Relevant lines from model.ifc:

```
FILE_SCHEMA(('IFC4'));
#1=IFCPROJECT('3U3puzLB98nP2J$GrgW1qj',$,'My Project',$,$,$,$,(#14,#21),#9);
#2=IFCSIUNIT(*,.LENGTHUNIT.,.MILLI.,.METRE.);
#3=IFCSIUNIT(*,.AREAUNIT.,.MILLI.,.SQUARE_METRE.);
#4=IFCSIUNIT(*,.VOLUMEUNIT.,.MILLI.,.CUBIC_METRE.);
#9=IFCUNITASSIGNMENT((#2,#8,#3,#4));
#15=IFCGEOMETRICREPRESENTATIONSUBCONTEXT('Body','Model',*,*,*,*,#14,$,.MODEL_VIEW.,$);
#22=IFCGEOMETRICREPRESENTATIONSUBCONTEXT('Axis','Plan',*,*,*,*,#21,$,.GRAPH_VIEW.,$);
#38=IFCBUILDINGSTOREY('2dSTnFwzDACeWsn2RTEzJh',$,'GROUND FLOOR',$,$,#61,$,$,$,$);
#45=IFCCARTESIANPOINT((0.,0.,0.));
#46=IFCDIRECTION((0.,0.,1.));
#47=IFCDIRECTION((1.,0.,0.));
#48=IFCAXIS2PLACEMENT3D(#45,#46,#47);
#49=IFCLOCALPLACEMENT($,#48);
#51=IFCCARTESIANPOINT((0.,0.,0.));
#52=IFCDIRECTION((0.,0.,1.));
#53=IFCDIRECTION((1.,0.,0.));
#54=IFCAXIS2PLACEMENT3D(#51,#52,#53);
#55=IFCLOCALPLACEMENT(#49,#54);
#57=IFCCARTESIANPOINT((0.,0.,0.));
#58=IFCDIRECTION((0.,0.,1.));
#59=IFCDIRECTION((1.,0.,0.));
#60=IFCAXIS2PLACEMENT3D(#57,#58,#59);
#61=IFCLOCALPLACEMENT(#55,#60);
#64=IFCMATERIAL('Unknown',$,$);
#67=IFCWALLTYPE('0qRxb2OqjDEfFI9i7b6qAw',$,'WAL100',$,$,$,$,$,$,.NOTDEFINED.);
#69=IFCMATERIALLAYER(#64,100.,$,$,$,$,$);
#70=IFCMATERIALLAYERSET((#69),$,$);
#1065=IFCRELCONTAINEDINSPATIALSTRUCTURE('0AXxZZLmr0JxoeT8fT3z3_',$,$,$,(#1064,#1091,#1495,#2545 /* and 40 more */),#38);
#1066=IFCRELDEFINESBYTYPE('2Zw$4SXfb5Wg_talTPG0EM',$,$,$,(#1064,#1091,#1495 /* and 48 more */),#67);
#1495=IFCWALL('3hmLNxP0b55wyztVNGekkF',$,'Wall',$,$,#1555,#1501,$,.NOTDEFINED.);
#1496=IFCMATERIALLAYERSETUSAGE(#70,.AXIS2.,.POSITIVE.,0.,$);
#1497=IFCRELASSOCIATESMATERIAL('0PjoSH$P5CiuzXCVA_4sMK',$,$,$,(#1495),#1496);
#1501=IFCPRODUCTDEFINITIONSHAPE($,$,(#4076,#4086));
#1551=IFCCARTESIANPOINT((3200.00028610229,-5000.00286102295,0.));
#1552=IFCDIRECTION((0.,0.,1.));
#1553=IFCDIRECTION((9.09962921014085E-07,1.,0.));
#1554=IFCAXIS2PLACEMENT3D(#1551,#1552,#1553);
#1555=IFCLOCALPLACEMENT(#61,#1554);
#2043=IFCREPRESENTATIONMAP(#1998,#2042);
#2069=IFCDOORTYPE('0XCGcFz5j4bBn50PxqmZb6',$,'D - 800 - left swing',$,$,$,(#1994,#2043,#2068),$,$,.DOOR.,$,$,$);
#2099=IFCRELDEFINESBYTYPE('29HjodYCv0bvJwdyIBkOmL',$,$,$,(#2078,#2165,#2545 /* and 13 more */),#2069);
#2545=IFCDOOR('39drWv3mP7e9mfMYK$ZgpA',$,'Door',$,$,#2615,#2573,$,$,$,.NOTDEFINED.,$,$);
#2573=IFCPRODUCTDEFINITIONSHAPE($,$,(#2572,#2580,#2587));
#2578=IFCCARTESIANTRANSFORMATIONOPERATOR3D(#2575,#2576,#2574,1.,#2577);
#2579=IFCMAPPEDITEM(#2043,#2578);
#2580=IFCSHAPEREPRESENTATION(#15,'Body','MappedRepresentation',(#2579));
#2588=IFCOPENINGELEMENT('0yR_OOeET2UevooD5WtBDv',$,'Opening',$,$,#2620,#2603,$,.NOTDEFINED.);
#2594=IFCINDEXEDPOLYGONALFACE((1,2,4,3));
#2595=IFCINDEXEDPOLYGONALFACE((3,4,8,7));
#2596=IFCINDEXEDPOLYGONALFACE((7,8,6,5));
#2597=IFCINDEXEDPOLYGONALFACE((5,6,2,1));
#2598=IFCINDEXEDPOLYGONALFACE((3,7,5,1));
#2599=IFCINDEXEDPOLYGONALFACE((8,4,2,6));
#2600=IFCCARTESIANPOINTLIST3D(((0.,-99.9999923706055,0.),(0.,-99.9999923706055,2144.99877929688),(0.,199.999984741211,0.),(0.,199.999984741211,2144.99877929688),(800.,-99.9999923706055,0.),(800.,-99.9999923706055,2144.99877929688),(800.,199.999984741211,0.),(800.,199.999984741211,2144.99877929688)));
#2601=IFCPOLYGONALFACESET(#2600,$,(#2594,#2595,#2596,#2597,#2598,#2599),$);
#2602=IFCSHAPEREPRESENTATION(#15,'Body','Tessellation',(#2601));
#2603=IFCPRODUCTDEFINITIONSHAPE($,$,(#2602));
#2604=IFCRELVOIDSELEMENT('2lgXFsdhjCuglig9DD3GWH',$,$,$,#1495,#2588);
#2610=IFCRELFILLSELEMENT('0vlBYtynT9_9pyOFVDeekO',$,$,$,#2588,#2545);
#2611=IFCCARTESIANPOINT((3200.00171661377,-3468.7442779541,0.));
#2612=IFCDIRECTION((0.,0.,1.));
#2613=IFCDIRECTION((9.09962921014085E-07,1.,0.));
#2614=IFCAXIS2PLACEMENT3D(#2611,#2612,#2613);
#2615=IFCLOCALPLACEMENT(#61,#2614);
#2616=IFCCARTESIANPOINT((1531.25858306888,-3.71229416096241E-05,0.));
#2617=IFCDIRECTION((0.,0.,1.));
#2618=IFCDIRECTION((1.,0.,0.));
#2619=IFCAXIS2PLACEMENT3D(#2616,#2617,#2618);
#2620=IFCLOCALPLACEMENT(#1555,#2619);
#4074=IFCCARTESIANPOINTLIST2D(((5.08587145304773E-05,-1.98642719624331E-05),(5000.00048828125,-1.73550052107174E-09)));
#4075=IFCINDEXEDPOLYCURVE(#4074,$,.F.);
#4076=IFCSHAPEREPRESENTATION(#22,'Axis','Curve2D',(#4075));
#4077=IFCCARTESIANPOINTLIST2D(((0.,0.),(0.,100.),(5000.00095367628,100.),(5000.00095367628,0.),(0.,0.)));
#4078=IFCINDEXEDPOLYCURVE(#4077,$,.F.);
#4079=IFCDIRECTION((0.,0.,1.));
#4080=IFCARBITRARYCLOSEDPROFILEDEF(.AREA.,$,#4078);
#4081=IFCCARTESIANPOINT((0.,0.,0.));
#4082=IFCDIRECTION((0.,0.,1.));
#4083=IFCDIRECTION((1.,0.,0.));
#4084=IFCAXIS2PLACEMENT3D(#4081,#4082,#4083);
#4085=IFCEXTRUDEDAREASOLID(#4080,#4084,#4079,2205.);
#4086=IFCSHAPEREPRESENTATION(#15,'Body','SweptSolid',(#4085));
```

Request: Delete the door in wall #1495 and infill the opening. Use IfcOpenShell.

```python
import ifcopenshell
import ifcopenshell.api.feature
import ifcopenshell.api.root
import ifcopenshell.geom
import ifcopenshell.util.shape

model = ifcopenshell.open("model.ifc")
settings = ifcopenshell.geom.settings()


def volume(element):
    """Net volume in cubic metres, openings subtracted."""
    shape = ifcopenshell.geom.create_shape(settings, element)
    return ifcopenshell.util.shape.get_volume(shape.geometry)


door = model.by_guid("39drWv3mP7e9mfMYK$ZgpA")
opening = door.FillsVoids[0].RelatingOpeningElement
wall = opening.VoidsElements[0].RelatingBuildingElement
before = volume(wall)

ifcopenshell.api.root.remove_product(model, product=door)
ifcopenshell.api.feature.remove_feature(model, feature=opening)

after = volume(wall)

print(f"wall volume {before:.3f} -> {after:.3f} m3")

model.write("model-out.ifc")
```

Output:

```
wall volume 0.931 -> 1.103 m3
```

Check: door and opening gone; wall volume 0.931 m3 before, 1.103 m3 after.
